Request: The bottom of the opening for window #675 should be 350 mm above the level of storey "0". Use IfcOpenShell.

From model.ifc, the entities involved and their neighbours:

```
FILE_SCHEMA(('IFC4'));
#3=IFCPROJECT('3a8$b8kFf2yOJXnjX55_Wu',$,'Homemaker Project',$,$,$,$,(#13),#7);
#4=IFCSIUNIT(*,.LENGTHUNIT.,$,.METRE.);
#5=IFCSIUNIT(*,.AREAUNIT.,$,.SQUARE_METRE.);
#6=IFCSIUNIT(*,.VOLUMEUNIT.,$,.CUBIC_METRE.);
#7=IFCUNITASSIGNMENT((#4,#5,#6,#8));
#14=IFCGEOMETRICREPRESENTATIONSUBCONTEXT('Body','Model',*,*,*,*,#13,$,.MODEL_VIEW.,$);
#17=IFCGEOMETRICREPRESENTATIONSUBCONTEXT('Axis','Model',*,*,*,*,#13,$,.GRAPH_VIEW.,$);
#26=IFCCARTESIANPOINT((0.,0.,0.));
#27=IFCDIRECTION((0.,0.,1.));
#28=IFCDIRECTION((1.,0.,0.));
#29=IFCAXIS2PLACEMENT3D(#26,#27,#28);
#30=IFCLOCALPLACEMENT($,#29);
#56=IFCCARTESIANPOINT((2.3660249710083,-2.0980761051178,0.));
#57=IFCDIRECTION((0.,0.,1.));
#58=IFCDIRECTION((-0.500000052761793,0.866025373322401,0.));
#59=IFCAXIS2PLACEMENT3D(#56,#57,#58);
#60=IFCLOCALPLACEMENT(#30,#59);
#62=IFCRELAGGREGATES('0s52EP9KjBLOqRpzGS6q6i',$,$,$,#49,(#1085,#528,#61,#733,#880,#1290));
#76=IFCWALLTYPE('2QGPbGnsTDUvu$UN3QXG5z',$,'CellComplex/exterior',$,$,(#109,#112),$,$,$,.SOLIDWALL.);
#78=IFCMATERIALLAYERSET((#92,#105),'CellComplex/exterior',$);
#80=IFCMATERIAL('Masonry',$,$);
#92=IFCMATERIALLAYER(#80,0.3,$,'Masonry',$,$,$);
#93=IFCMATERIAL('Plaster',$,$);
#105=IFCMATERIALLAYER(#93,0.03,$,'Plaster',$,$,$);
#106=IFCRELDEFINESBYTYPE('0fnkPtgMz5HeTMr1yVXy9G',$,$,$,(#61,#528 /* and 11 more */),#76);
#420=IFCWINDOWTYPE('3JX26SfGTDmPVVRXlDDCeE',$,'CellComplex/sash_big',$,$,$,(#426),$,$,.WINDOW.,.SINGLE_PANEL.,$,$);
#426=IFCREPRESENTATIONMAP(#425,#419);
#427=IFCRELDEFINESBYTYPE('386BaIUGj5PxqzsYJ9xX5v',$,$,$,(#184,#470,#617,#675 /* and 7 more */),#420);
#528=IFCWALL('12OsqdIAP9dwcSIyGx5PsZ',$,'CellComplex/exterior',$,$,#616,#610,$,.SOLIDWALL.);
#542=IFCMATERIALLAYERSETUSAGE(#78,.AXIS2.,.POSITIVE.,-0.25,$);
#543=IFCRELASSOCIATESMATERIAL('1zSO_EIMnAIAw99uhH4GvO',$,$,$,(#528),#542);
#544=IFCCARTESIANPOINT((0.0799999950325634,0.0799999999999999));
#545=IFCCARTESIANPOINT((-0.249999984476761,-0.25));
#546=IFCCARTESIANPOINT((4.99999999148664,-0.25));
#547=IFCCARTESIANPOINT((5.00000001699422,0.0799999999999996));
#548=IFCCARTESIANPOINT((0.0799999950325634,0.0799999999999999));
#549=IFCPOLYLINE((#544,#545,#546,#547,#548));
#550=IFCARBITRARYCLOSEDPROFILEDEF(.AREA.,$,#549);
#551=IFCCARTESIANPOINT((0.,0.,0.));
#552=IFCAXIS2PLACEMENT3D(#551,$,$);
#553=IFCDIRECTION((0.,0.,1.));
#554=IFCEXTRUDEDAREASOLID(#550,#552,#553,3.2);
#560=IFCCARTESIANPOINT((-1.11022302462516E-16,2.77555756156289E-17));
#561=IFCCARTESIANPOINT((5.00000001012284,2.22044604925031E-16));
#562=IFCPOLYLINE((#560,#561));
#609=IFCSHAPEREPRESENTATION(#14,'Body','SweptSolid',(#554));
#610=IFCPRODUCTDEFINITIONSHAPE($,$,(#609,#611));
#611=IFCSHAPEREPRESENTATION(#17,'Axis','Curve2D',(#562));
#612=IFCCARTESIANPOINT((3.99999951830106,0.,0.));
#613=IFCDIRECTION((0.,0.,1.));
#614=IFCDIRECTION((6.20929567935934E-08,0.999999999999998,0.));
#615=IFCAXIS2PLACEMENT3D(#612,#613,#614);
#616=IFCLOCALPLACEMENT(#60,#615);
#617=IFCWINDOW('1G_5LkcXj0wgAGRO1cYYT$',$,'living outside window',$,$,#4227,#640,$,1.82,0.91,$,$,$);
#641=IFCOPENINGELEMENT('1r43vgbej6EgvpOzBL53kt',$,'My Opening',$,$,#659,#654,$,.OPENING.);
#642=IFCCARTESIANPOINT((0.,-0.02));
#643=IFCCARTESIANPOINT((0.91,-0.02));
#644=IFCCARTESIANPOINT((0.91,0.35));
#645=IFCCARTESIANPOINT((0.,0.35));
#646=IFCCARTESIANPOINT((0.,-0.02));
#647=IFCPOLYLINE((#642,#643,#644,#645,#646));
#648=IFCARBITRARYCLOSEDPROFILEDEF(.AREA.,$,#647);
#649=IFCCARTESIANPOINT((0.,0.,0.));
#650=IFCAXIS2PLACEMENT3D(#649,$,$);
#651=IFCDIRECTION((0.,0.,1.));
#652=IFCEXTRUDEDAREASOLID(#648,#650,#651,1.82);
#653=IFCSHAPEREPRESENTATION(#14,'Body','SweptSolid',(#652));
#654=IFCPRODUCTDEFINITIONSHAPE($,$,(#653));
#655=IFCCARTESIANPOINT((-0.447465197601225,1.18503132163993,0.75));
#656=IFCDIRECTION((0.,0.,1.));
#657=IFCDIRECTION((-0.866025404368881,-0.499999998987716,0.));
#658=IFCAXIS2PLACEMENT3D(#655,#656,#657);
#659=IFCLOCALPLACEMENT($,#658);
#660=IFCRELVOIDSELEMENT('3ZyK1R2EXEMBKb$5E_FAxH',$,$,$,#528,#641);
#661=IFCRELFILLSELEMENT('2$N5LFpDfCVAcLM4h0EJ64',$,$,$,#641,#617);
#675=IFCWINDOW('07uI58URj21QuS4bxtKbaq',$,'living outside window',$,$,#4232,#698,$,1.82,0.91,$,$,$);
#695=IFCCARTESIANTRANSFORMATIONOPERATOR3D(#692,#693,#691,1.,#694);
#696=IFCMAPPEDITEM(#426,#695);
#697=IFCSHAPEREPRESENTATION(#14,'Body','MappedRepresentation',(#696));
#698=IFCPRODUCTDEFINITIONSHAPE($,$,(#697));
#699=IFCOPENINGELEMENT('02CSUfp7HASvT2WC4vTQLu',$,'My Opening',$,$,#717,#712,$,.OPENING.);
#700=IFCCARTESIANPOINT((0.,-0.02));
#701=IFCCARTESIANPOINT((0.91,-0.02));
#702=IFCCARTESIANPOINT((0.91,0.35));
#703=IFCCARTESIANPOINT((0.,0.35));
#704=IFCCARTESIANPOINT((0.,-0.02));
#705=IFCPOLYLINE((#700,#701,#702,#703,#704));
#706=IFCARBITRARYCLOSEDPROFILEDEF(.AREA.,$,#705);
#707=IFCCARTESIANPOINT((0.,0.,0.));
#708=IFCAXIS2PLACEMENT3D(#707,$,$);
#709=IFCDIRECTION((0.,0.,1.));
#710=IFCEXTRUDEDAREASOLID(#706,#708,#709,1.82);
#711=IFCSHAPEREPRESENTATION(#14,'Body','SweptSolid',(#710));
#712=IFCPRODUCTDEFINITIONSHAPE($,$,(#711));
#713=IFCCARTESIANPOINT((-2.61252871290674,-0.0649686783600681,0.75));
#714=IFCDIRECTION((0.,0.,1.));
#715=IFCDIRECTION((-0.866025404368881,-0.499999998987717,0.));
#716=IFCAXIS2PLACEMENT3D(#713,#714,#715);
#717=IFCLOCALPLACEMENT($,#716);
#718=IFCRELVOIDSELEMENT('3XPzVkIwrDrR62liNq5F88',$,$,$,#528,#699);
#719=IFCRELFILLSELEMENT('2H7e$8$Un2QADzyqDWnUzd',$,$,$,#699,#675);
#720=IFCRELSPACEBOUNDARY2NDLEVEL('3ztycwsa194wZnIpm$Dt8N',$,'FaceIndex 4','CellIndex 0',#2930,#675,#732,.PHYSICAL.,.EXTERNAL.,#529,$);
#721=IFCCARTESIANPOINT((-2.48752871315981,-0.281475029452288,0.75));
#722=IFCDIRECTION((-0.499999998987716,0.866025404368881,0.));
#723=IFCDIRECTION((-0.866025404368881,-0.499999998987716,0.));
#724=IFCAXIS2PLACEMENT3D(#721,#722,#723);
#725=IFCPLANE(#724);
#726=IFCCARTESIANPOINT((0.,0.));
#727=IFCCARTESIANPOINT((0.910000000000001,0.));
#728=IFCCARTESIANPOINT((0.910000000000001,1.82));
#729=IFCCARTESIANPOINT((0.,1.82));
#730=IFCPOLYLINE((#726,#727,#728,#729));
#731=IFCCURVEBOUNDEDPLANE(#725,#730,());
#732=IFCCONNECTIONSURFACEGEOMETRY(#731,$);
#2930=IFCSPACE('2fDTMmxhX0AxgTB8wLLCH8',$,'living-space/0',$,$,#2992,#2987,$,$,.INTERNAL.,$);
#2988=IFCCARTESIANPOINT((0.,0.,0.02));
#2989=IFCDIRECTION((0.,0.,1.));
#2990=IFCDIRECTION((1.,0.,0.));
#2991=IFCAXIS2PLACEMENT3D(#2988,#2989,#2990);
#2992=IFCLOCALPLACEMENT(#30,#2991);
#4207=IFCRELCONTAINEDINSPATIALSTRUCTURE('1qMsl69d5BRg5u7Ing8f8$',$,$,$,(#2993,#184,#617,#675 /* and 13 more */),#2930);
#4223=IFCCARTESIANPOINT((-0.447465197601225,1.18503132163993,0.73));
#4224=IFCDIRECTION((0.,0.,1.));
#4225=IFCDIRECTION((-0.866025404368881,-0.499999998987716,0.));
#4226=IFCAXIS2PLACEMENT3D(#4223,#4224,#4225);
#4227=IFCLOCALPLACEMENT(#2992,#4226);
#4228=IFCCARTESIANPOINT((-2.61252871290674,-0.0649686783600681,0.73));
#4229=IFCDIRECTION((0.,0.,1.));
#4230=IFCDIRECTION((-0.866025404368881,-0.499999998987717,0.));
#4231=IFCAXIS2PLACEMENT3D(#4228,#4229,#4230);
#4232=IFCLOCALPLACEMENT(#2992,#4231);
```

```python
import numpy as np
import ifcopenshell
import ifcopenshell.api.geometry
import ifcopenshell.geom
import ifcopenshell.util.element
import ifcopenshell.util.placement
import ifcopenshell.util.shape
import ifcopenshell.util.unit

model = ifcopenshell.open("model.ifc")
unit_scale = ifcopenshell.util.unit.calculate_unit_scale(model)

window = model.by_guid("07uI58URj21QuS4bxtKbaq")
opening = window.FillsVoids[0].RelatingOpeningElement
storey = ifcopenshell.util.element.get_container(window, ifc_class="IfcBuildingStorey")
level = ifcopenshell.util.placement.get_local_placement(storey.ObjectPlacement)[2, 3]

# The opening's origin need not be at the sill, so measure its lowest point.
shape = ifcopenshell.geom.create_shape(ifcopenshell.geom.settings(), opening)
bottom = ifcopenshell.util.shape.get_shape_bottom_elevation(shape, shape.geometry) / unit_scale
dz = level + 0.35 - bottom

shift = np.array([0.0, 0.0, dz])
# The window is not placed relative to its opening, so move both.
for product in (opening, window):
    matrix = ifcopenshell.util.placement.get_local_placement(product.ObjectPlacement)
    matrix[:3, 3] += shift
    ifcopenshell.api.geometry.edit_object_placement(model, product=product, matrix=matrix, is_si=False)

# Space boundary surfaces are stored in each space's coordinates; move them too.
for rel in window.ProvidesBoundaries:
    if not rel.ConnectionGeometry:
        continue
    surface = rel.ConnectionGeometry.SurfaceOnRelatingElement.BasisSurface
    space_matrix = ifcopenshell.util.placement.get_local_placement(rel.RelatingSpace.ObjectPlacement)
    point = np.array(surface.Position.Location.Coordinates) + space_matrix[:3, :3].T @ shift
    surface.Position = model.createIfcAxis2Placement3D(
        model.createIfcCartesianPoint(point.tolist()), surface.Position.Axis, surface.Position.RefDirection
    )

print(f"moved by {dz * unit_scale:+.3f} m")

model.write("model_updated.ifc")
```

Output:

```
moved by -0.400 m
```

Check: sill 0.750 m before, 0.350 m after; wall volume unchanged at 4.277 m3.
